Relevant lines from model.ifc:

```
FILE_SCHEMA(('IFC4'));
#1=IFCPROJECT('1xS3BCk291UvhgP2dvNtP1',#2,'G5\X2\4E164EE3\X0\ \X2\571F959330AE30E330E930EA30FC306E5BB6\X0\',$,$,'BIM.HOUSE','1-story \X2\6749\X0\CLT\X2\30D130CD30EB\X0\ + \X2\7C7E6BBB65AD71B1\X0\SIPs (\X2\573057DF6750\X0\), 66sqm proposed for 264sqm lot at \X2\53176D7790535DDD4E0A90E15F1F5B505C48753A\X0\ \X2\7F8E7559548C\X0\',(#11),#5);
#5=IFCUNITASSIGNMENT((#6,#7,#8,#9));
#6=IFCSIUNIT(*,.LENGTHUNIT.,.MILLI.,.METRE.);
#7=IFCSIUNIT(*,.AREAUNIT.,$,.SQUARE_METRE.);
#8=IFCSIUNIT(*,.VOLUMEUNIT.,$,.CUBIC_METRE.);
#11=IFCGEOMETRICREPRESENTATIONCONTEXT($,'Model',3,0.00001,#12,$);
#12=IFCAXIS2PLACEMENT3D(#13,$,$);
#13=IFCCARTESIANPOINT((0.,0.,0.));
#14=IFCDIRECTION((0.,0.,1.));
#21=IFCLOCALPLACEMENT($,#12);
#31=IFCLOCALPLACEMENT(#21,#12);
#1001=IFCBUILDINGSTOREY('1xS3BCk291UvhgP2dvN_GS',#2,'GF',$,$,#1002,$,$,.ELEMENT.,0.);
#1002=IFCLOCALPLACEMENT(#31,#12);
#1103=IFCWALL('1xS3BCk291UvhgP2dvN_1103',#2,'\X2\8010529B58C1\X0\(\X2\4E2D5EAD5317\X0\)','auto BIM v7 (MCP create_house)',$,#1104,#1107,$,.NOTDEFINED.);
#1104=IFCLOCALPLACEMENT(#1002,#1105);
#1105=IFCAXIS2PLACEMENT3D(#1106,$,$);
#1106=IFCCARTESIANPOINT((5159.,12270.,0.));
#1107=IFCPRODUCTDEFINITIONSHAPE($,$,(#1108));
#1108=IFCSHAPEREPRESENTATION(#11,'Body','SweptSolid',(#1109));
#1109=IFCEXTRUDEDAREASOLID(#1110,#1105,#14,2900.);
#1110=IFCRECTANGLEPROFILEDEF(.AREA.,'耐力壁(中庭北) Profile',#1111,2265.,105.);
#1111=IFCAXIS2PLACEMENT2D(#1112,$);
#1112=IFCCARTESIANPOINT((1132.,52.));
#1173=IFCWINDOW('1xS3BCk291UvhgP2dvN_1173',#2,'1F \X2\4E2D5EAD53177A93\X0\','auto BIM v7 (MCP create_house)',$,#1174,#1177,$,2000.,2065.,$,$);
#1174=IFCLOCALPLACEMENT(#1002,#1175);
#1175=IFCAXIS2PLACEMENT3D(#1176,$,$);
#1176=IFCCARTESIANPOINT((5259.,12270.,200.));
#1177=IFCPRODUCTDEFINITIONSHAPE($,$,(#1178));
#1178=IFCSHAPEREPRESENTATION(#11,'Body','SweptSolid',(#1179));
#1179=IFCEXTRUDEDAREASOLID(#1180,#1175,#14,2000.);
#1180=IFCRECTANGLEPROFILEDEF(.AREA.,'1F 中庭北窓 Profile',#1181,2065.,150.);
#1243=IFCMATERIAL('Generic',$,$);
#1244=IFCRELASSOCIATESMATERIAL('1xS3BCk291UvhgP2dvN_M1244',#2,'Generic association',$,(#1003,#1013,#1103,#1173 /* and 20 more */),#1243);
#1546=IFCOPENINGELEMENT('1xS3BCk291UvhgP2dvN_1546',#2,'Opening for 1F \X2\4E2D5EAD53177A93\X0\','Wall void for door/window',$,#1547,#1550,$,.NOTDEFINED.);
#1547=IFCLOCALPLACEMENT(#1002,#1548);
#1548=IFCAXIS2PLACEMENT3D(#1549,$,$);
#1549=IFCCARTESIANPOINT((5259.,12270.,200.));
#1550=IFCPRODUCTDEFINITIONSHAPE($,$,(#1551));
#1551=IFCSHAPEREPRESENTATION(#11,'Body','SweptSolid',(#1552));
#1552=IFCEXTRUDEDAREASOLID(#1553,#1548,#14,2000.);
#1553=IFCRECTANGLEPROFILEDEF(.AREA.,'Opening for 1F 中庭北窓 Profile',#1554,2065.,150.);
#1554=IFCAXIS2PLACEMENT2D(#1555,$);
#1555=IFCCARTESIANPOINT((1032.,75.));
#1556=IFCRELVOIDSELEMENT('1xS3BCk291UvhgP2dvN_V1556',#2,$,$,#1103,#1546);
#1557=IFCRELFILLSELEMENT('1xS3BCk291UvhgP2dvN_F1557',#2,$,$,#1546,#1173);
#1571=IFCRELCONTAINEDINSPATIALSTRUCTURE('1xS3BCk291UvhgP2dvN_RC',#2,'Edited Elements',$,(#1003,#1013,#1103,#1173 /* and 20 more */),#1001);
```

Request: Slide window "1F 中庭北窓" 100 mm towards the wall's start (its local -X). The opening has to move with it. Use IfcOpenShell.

```python
import ifcopenshell
import ifcopenshell.api.geometry
import ifcopenshell.util.placement
import ifcopenshell.util.unit

model = ifcopenshell.open("model.ifc")
unit_scale = ifcopenshell.util.unit.calculate_unit_scale(model)

window = model.by_id(1173)
opening = window.FillsVoids[0].RelatingOpeningElement
wall = opening.VoidsElements[0].RelatingBuildingElement

wall_matrix = ifcopenshell.util.placement.get_local_placement(wall.ObjectPlacement)
shift = wall_matrix[:3, 0] * -0.1 / unit_scale
before = ifcopenshell.util.placement.get_local_placement(window.ObjectPlacement)[:3, 3].copy()

# The window is not placed relative to its opening, so move both.
for product in (opening, window):
    matrix = ifcopenshell.util.placement.get_local_placement(product.ObjectPlacement)
    matrix[:3, 3] += shift
    ifcopenshell.api.geometry.edit_object_placement(model, product=product, matrix=matrix, is_si=False)

after = ifcopenshell.util.placement.get_local_placement(window.ObjectPlacement)[:3, 3]
print("window moved by", (after - before).round(3) + 0.0)

model.write("model_v2.ifc")
```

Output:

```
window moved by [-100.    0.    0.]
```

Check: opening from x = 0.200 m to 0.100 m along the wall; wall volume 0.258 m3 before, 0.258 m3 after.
